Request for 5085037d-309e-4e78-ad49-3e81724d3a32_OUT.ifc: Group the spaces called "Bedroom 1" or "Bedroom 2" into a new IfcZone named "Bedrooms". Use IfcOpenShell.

First a look at what the model holds.

```python
import ifcopenshell

model = ifcopenshell.open("5085037d-309e-4e78-ad49-3e81724d3a32_OUT.ifc")
print(model.schema)
seen = {}
for space in model.by_type("IfcSpace"):
    seen[space.LongName] = seen.get(space.LongName, 0) + 1
for name, count in sorted(seen.items(), key=str):
    print(count, "x", name)
print("zones:", [z.Name for z in model.by_type("IfcZone")][:20])
```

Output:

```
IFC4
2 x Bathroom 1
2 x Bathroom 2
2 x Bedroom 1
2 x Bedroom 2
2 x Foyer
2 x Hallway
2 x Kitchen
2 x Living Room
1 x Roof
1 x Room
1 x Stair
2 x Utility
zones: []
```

```python
import ifcopenshell
import ifcopenshell.api.group
import ifcopenshell.api.root

model = ifcopenshell.open("5085037d-309e-4e78-ad49-3e81724d3a32_OUT.ifc")

names = {"Bedroom 1", "Bedroom 2"}
spaces = [s for s in model.by_type("IfcSpace") if s.LongName in names]

zone = ifcopenshell.api.root.create_entity(model, ifc_class="IfcZone", name="Bedrooms")
ifcopenshell.api.group.assign_group(model, products=spaces, group=zone)
print(len(spaces), "spaces in", zone.Name)

model.write("5085037d-309e-4e78-ad49-3e81724d3a32_OUT_updated.ifc")
```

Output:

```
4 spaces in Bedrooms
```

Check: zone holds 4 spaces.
